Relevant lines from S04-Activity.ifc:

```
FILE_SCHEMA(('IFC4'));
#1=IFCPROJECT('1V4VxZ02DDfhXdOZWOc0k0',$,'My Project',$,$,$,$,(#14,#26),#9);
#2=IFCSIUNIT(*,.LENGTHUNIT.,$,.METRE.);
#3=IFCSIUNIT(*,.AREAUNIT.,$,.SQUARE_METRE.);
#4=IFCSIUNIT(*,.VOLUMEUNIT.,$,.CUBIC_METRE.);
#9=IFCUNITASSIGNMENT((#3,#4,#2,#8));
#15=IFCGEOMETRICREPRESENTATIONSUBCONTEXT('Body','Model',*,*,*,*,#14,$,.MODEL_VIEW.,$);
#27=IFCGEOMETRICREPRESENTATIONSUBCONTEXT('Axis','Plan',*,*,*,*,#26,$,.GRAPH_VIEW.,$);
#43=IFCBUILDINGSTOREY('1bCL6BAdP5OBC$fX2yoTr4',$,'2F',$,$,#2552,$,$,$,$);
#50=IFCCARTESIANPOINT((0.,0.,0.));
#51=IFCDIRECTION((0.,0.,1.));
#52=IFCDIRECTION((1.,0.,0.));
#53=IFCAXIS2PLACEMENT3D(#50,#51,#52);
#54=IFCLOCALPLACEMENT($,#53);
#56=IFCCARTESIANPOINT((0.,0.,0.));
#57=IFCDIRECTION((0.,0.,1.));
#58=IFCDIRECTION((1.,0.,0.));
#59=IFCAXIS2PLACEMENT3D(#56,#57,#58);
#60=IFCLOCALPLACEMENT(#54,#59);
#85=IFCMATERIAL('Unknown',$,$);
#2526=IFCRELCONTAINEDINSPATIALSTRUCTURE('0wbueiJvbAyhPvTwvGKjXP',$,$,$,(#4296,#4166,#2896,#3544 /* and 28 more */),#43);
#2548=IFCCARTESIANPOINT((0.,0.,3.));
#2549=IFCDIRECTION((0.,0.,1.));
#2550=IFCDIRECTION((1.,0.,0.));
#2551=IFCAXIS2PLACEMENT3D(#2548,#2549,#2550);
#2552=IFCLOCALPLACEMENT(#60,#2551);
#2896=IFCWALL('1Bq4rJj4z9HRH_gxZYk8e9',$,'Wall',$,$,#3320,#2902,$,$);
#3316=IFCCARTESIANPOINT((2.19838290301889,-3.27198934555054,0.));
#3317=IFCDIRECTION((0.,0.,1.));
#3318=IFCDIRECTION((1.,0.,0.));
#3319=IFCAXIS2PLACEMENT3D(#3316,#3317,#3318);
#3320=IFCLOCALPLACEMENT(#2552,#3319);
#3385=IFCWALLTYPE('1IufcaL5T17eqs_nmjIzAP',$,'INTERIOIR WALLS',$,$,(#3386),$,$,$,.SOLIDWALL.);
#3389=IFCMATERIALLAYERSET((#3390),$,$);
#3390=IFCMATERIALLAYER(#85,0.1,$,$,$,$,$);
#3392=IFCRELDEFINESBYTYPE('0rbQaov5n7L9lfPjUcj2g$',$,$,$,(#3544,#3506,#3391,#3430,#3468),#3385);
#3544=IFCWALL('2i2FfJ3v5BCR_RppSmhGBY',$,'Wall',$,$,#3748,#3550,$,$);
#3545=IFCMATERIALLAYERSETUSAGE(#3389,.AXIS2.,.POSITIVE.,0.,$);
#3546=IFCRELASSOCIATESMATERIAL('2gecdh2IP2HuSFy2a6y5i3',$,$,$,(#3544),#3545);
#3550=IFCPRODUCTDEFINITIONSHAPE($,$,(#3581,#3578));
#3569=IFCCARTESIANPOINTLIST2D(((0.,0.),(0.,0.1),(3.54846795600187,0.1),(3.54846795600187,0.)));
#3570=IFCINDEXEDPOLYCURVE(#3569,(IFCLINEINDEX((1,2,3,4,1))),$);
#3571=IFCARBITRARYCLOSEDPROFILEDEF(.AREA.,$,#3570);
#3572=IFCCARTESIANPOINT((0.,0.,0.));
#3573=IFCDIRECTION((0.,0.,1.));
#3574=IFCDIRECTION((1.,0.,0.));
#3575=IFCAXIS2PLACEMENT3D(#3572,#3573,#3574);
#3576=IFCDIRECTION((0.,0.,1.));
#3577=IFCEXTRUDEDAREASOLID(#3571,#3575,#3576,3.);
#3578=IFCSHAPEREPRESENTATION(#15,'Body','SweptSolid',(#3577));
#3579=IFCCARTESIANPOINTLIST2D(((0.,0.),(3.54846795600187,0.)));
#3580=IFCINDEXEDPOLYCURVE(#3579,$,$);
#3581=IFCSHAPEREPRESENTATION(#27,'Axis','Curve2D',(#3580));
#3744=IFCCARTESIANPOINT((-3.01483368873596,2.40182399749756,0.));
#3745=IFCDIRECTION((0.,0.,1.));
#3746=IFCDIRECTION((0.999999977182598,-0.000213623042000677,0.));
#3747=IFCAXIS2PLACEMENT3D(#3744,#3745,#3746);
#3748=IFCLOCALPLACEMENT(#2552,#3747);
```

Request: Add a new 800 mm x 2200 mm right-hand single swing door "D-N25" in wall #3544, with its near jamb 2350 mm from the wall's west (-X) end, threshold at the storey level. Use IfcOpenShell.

```python
import numpy as np
import ifcopenshell
import ifcopenshell.api.feature
import ifcopenshell.api.geometry
import ifcopenshell.api.root
import ifcopenshell.api.spatial
import ifcopenshell.geom
import ifcopenshell.util.element
import ifcopenshell.util.placement
import ifcopenshell.util.representation
import ifcopenshell.util.shape
import ifcopenshell.util.unit

model = ifcopenshell.open("S04-Activity.ifc")
unit_scale = ifcopenshell.util.unit.calculate_unit_scale(model)
settings = ifcopenshell.geom.settings()


def volume(element):
    """Net volume in cubic metres, openings subtracted."""
    shape = ifcopenshell.geom.create_shape(settings, element)
    return ifcopenshell.util.shape.get_volume(shape.geometry)


wall = model.by_id(3544)
storey = ifcopenshell.util.element.get_container(wall, ifc_class="IfcBuildingStorey")
context = ifcopenshell.util.representation.get_context(model, "Model", "Body", "MODEL_VIEW")
before = volume(wall)

width, height, from_end, sill = 0.8, 2.2, 2.35, 0.0  # metres

# The wall runs along its own X axis, and the end named is its -X end.
wall_shape = ifcopenshell.geom.create_shape(settings, wall)
x, y, z = ifcopenshell.util.shape.get_vertices(wall_shape.geometry).T
start = x.min() + from_end
face, thickness = float(y.min()), float(y.max() - y.min())
wall_matrix = ifcopenshell.util.placement.get_local_placement(wall.ObjectPlacement)
level = ifcopenshell.util.placement.get_local_placement(storey.ObjectPlacement)[2, 3]


def in_wall(x, y):
    """Placement at x, y metres in the wall's axes, at sill height."""
    matrix = wall_matrix.copy()
    matrix[:, 3] = wall_matrix @ np.array([x / unit_scale, y / unit_scale, 0.0, 1.0])
    matrix[2, 3] = level + sill / unit_scale
    return matrix


# Opening: a box that overshoots both wall faces by 50 mm.
opening = ifcopenshell.api.root.create_entity(model, ifc_class="IfcOpeningElement", predefined_type="OPENING")
box = ifcopenshell.api.geometry.add_wall_representation(
    model, context=context, length=width, height=height, thickness=thickness + 0.1
)
ifcopenshell.api.geometry.assign_representation(model, product=opening, representation=box)
ifcopenshell.api.geometry.edit_object_placement(model, product=opening, matrix=in_wall(start, face - 0.05), is_si=False)
ifcopenshell.api.feature.add_feature(model, feature=opening, element=wall)

door = ifcopenshell.api.root.create_entity(model, ifc_class="IfcDoor", name="D-N25", predefined_type="DOOR")
door.OverallWidth, door.OverallHeight = width / unit_scale, height / unit_scale
door.OperationType = "SINGLE_SWING_RIGHT"
body = ifcopenshell.api.geometry.add_door_representation(
    model,
    context=context,
    overall_width=door.OverallWidth,
    overall_height=door.OverallHeight,
    operation_type="SINGLE_SWING_RIGHT",
    lining_properties={"LiningDepth": thickness / unit_scale, "ThresholdDepth": thickness / unit_scale},
)
ifcopenshell.api.geometry.assign_representation(model, product=door, representation=body)
ifcopenshell.api.spatial.assign_container(model, products=[door], relating_structure=storey)
ifcopenshell.api.feature.add_filling(model, opening=opening, element=door)

# The lining spans the wall, so the door starts at the wall face.
ifcopenshell.api.geometry.edit_object_placement(model, product=door, matrix=in_wall(start, face), is_si=False)

after = volume(wall)

print(f"wall volume {before:.3f} -> {after:.3f} m3")

model.write("S04-Activity_updated.ifc")
```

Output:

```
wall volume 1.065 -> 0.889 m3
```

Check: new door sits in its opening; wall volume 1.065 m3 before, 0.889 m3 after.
